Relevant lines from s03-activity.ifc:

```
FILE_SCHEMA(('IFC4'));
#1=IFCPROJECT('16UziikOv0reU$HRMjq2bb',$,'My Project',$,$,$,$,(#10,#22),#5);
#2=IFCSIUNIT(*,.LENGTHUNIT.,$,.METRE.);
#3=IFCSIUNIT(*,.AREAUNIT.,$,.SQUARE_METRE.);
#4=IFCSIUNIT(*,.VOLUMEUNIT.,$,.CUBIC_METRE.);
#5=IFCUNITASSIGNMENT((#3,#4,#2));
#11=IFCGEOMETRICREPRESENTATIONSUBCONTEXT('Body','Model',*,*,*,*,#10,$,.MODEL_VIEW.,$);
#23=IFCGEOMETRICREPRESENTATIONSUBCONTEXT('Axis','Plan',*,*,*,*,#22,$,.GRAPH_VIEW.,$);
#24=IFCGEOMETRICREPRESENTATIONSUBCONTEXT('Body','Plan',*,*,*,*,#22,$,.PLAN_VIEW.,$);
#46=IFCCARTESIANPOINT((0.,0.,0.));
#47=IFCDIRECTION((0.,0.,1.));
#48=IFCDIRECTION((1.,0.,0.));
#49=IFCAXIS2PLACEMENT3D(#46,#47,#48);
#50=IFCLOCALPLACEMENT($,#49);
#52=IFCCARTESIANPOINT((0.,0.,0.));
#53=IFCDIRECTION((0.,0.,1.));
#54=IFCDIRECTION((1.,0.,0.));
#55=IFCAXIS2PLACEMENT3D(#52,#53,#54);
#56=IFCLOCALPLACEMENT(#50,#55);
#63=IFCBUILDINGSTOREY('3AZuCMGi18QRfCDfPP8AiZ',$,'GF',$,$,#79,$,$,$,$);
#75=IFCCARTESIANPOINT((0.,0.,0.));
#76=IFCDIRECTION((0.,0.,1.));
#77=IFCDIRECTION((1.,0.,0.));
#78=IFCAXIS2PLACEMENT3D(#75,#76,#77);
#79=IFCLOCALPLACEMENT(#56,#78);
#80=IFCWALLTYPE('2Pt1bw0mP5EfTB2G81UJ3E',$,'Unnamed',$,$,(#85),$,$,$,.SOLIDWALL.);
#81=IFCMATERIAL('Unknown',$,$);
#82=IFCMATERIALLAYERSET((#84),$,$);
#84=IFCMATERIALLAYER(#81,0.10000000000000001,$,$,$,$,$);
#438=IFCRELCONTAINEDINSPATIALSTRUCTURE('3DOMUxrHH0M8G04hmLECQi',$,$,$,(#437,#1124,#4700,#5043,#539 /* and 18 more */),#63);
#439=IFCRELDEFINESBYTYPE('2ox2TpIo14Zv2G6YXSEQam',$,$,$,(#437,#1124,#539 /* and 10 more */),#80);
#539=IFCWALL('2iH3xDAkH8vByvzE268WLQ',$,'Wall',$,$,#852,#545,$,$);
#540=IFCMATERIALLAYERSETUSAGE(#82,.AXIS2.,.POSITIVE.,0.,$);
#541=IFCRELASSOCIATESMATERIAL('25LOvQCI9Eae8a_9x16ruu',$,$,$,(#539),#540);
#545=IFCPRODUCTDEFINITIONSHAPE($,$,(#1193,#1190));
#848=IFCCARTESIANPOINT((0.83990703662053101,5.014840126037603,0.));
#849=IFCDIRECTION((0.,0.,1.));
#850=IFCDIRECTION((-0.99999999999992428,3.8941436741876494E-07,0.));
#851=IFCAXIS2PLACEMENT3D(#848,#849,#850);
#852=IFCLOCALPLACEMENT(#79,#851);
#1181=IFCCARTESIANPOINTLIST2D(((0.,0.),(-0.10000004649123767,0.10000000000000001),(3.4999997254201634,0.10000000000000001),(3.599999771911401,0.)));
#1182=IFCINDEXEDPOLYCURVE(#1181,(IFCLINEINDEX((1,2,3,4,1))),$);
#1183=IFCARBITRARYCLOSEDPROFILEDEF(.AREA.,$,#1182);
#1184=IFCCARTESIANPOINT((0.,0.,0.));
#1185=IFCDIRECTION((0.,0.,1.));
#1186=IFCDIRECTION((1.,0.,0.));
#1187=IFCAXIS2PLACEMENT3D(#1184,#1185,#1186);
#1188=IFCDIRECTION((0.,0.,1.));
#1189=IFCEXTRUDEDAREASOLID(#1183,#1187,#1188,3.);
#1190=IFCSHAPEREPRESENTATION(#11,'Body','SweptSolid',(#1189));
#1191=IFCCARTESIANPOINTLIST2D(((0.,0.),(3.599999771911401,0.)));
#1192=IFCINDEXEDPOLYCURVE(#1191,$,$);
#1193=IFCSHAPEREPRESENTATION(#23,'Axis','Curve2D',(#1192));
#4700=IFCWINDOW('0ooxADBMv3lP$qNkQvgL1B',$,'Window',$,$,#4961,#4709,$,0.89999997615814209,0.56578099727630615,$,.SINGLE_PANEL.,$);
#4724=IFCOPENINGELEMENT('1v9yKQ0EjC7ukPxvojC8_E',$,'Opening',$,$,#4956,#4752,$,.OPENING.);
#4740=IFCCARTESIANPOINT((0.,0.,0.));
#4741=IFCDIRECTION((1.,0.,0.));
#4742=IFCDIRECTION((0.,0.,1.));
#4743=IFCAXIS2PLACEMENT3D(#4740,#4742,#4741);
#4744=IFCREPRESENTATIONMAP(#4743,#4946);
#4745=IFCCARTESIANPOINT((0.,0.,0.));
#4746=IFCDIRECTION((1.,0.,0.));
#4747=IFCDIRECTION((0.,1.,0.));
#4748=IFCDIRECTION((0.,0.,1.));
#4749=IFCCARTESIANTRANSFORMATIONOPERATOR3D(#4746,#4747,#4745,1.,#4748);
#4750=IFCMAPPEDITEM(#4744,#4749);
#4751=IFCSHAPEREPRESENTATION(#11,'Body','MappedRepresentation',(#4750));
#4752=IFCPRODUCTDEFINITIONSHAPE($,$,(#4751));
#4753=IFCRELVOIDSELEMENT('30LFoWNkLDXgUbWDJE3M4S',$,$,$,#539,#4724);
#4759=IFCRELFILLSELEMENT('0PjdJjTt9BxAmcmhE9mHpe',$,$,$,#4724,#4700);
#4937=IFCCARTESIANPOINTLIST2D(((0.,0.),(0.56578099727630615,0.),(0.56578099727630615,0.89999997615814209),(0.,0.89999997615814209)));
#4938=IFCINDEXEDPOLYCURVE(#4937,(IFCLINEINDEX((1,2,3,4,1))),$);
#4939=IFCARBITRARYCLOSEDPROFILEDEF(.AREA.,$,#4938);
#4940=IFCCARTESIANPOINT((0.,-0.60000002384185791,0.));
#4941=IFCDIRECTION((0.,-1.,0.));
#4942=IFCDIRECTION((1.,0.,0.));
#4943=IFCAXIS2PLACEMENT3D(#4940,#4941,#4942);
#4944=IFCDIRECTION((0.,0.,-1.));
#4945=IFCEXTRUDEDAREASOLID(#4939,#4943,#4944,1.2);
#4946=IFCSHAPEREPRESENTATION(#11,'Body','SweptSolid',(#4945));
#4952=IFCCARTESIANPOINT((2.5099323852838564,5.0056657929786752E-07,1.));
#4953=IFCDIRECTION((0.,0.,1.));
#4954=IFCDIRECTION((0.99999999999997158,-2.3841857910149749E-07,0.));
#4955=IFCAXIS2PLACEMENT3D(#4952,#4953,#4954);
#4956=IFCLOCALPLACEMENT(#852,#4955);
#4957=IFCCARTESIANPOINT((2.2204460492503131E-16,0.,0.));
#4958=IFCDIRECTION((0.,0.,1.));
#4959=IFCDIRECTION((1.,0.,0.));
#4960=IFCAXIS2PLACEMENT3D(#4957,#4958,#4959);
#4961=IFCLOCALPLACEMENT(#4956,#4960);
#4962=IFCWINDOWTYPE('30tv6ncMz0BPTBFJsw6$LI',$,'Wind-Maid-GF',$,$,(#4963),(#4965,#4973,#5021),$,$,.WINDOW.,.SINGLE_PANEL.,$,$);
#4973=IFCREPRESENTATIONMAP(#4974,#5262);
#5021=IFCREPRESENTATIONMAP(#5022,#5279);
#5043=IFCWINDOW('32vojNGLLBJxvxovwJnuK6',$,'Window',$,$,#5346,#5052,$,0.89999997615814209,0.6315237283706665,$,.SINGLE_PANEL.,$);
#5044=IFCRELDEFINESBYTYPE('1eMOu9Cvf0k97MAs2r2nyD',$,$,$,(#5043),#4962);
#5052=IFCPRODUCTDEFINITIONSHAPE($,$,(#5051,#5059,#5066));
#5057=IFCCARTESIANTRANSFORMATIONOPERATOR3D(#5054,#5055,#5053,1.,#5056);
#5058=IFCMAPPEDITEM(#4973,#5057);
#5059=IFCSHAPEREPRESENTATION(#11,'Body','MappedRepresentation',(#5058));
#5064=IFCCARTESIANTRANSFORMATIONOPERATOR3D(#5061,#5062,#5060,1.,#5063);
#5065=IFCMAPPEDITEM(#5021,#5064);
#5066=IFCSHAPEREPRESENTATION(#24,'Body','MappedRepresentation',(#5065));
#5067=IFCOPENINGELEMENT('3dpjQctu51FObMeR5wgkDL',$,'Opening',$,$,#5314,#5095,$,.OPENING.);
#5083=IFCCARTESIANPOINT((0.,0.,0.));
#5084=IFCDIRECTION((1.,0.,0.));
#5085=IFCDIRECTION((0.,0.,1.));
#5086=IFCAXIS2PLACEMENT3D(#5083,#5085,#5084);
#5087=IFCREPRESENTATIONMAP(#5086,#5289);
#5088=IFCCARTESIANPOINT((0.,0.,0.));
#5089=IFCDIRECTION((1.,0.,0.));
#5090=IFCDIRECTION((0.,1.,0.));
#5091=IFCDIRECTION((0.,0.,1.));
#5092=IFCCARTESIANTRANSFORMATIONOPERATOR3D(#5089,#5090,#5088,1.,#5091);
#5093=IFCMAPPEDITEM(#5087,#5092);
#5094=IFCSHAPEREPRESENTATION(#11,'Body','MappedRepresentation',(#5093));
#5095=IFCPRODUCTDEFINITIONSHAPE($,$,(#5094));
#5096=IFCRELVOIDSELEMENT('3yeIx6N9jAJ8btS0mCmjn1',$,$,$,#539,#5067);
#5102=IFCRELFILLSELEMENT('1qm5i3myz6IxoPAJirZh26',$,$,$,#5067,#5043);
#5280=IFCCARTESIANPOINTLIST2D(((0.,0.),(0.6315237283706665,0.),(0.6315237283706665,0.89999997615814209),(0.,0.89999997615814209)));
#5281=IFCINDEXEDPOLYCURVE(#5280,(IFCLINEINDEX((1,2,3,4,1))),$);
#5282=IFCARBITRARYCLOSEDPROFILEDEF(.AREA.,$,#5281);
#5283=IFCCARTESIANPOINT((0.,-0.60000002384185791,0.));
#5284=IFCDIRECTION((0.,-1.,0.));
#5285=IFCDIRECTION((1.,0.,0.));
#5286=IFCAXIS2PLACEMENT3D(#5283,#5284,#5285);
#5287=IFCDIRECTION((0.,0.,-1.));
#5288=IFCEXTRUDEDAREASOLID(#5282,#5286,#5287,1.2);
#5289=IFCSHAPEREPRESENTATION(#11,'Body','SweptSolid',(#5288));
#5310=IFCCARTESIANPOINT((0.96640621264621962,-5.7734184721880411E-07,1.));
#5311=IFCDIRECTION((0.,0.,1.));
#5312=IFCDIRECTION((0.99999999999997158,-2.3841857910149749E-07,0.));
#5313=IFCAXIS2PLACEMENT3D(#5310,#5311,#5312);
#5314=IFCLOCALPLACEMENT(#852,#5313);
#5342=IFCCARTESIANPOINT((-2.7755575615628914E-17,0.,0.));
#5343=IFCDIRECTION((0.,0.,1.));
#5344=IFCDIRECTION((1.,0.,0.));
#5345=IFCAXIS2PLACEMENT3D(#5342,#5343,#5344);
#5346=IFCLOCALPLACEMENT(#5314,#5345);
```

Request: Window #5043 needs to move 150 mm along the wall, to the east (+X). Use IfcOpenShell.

```python
import ifcopenshell
import ifcopenshell.api.geometry
import ifcopenshell.util.placement
import ifcopenshell.util.unit

model = ifcopenshell.open("s03-activity.ifc")
unit_scale = ifcopenshell.util.unit.calculate_unit_scale(model)

window = model.by_guid("32vojNGLLBJxvxovwJnuK6")
opening = window.FillsVoids[0].RelatingOpeningElement
wall = opening.VoidsElements[0].RelatingBuildingElement

wall_matrix = ifcopenshell.util.placement.get_local_placement(wall.ObjectPlacement)
shift = wall_matrix[:3, 0] * -0.15 / unit_scale
before = ifcopenshell.util.placement.get_local_placement(window.ObjectPlacement)[:3, 3].copy()

# The window is placed relative to its opening, so it follows when the opening moves.
matrix = ifcopenshell.util.placement.get_local_placement(opening.ObjectPlacement)
matrix[:3, 3] += shift
ifcopenshell.api.geometry.edit_object_placement(
    model, product=opening, matrix=matrix, is_si=False, should_transform_children=True
)

after = ifcopenshell.util.placement.get_local_placement(window.ObjectPlacement)[:3, 3]
print("window moved by", (after - before).round(3) + 0.0)

model.write("s03-activity-out.ifc")
```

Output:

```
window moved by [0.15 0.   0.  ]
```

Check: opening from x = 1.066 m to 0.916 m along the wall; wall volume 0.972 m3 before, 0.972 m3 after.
